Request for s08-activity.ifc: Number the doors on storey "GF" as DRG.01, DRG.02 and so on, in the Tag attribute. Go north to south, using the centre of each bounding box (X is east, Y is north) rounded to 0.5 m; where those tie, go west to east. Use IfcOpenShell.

First a look at what the model holds.

```python
import ifcopenshell
import ifcopenshell.util.element
import ifcopenshell.util.placement

model = ifcopenshell.open("s08-activity.ifc")
print(model.schema)
storey = next(s for s in model.by_type("IfcBuildingStorey") if s.Name == "GF")
doors = [e for e in ifcopenshell.util.element.get_decomposition(storey) if e.is_a("IfcDoor")]
for e in sorted(doors, key=lambda e: e.id()):
    origin = ifcopenshell.util.placement.get_local_placement(e.ObjectPlacement)[:3, 3]
    print(e.id(), e.Tag, e.Name, origin.round(2) + 0.0, sep=" | ")
```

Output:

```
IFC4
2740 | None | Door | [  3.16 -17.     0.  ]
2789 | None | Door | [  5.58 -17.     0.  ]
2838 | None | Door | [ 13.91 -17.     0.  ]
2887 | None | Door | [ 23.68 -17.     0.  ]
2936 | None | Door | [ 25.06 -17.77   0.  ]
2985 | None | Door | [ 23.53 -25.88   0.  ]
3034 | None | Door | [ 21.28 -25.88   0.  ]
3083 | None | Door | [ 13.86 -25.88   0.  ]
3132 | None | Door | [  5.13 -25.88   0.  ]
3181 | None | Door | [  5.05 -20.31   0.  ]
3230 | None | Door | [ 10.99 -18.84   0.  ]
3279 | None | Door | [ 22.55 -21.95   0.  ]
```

```python
import ifcopenshell
import ifcopenshell.geom
import ifcopenshell.util.element
import ifcopenshell.util.shape

model = ifcopenshell.open("s08-activity.ifc")
settings = ifcopenshell.geom.settings()
settings.set("use-world-coords", True)


def centre(element):
    shape = ifcopenshell.geom.create_shape(settings, element)
    return ifcopenshell.util.shape.get_bbox_centroid(shape.geometry)


storey = next(s for s in model.by_type("IfcBuildingStorey") if s.Name == "GF")
doors = [e for e in ifcopenshell.util.element.get_decomposition(storey) if e.is_a("IfcDoor")]

# Insertion points can sit at a corner or the storey origin, so sort by the geometry (in metres).
centres = {e: centre(e) for e in doors}
doors.sort(key=lambda e: (-round(centres[e][1] / 0.5), centres[e][0]))

for i, e in enumerate(doors, start=1):
    number = f"DRG.{i:02d}"
    e.Tag = number
    print(e.id(), number)

model.write("s08-activity_rev.ifc")
```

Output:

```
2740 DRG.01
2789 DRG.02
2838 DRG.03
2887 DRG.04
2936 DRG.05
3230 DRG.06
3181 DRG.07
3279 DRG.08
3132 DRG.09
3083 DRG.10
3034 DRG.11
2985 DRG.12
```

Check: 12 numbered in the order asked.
